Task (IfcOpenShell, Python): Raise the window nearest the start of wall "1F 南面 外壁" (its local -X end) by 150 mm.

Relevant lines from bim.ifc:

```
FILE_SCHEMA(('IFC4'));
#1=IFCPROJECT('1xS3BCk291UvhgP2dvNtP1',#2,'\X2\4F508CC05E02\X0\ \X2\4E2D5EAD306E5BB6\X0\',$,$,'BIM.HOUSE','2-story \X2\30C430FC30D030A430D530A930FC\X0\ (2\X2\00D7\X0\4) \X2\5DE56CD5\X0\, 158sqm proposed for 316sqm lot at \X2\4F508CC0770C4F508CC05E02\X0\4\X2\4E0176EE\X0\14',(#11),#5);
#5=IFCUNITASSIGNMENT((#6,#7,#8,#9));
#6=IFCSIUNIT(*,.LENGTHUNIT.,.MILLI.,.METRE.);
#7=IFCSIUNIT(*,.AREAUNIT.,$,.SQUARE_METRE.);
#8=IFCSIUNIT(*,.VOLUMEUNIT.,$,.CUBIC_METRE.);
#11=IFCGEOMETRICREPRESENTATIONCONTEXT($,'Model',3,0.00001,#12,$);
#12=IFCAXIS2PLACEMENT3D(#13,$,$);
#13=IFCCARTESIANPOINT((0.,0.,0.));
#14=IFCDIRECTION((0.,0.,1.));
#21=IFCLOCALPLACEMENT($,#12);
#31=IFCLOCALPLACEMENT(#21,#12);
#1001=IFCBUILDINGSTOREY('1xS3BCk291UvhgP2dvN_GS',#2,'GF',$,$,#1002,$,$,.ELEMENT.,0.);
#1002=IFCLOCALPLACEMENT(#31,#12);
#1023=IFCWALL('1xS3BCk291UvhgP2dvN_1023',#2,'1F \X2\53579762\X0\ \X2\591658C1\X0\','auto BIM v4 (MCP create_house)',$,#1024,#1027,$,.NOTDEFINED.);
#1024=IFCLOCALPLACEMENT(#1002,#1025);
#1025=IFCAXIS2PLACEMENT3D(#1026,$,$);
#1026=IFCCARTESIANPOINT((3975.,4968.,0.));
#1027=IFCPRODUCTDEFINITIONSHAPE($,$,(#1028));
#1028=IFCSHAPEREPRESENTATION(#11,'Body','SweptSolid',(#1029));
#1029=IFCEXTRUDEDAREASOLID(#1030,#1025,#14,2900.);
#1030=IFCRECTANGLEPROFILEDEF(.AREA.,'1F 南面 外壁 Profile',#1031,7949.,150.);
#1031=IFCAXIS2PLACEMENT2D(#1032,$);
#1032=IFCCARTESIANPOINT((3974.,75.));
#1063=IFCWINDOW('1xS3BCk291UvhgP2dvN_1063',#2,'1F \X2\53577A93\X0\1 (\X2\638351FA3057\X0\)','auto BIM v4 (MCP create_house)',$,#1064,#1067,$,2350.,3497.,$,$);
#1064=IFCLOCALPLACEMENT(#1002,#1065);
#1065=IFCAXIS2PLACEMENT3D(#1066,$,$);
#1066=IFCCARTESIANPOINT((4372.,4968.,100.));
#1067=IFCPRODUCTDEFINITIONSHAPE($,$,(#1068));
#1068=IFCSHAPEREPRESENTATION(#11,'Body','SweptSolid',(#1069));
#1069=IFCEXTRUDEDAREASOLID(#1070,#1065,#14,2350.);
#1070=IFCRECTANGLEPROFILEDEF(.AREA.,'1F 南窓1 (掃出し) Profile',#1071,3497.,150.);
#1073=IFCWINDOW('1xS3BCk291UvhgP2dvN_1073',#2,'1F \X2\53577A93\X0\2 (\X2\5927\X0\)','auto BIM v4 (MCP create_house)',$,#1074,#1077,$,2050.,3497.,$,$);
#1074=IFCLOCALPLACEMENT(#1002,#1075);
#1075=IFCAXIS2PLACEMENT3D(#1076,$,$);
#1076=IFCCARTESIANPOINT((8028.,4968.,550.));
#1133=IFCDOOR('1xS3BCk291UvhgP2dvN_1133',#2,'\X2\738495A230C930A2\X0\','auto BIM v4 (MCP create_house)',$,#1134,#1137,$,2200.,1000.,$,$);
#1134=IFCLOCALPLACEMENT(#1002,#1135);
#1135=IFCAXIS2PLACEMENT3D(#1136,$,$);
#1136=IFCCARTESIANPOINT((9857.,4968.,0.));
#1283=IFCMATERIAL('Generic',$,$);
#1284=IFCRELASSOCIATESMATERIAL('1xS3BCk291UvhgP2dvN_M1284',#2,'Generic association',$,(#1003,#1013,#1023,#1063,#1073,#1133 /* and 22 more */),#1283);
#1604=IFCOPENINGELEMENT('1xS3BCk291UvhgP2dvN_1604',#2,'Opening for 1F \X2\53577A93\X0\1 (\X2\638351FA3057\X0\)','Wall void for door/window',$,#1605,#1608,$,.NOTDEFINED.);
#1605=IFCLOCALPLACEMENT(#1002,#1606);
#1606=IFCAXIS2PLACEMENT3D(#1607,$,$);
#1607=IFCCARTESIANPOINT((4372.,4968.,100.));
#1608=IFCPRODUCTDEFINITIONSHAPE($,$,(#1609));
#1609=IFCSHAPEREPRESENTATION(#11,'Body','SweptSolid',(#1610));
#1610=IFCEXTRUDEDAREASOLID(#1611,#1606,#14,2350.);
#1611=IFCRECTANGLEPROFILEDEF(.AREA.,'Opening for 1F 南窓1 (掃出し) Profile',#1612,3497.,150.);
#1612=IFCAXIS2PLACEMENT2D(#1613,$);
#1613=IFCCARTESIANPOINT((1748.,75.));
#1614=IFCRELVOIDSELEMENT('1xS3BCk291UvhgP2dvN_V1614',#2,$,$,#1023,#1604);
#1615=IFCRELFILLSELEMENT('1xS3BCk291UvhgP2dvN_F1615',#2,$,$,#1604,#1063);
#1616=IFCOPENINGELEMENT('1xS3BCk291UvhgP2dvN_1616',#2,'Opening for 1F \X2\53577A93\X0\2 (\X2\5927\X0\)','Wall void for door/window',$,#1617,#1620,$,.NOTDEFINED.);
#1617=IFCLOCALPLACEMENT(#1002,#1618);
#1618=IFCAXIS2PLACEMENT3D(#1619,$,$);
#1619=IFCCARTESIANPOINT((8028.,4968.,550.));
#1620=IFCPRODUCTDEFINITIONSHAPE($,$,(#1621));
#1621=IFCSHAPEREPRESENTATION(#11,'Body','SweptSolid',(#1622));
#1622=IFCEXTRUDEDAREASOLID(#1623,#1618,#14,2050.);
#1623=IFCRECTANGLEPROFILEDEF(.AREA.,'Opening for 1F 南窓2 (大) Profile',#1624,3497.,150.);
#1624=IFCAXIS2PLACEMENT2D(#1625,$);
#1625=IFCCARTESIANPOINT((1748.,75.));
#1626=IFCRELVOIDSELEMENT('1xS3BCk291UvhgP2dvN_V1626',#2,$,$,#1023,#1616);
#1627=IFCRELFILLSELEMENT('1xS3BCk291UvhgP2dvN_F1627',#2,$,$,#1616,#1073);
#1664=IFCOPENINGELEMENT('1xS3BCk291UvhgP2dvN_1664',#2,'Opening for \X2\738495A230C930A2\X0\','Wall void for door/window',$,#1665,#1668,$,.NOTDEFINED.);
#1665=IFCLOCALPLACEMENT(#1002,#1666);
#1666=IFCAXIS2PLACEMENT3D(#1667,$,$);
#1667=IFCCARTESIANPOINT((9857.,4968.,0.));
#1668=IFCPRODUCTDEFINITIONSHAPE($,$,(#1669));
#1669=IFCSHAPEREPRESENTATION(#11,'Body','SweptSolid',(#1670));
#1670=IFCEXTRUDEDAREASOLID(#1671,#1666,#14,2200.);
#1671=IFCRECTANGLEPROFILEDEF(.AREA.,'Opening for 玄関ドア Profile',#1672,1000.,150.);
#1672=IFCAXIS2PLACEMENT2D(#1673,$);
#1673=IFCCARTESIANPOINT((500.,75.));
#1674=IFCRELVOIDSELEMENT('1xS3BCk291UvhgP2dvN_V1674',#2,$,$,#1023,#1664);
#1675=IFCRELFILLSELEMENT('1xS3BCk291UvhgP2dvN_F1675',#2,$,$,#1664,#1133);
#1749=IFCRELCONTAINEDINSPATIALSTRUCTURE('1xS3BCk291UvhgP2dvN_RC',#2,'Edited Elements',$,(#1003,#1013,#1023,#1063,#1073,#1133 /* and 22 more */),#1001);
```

```python
import numpy as np
import ifcopenshell
import ifcopenshell.api.geometry
import ifcopenshell.util.placement
import ifcopenshell.util.unit

model = ifcopenshell.open("bim.ifc")
unit_scale = ifcopenshell.util.unit.calculate_unit_scale(model)

window = model.by_guid("1xS3BCk291UvhgP2dvN_1063")
opening = window.FillsVoids[0].RelatingOpeningElement
dz = 0.15 / unit_scale

shift = np.array([0.0, 0.0, dz])
# The window is not placed relative to its opening, so move both.
for product in (opening, window):
    matrix = ifcopenshell.util.placement.get_local_placement(product.ObjectPlacement)
    matrix[:3, 3] += shift
    ifcopenshell.api.geometry.edit_object_placement(model, product=product, matrix=matrix, is_si=False)

print(f"moved by {dz * unit_scale:+.3f} m")

model.write("bim_edited.ifc")
```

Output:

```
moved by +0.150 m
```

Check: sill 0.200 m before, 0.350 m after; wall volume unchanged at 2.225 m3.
